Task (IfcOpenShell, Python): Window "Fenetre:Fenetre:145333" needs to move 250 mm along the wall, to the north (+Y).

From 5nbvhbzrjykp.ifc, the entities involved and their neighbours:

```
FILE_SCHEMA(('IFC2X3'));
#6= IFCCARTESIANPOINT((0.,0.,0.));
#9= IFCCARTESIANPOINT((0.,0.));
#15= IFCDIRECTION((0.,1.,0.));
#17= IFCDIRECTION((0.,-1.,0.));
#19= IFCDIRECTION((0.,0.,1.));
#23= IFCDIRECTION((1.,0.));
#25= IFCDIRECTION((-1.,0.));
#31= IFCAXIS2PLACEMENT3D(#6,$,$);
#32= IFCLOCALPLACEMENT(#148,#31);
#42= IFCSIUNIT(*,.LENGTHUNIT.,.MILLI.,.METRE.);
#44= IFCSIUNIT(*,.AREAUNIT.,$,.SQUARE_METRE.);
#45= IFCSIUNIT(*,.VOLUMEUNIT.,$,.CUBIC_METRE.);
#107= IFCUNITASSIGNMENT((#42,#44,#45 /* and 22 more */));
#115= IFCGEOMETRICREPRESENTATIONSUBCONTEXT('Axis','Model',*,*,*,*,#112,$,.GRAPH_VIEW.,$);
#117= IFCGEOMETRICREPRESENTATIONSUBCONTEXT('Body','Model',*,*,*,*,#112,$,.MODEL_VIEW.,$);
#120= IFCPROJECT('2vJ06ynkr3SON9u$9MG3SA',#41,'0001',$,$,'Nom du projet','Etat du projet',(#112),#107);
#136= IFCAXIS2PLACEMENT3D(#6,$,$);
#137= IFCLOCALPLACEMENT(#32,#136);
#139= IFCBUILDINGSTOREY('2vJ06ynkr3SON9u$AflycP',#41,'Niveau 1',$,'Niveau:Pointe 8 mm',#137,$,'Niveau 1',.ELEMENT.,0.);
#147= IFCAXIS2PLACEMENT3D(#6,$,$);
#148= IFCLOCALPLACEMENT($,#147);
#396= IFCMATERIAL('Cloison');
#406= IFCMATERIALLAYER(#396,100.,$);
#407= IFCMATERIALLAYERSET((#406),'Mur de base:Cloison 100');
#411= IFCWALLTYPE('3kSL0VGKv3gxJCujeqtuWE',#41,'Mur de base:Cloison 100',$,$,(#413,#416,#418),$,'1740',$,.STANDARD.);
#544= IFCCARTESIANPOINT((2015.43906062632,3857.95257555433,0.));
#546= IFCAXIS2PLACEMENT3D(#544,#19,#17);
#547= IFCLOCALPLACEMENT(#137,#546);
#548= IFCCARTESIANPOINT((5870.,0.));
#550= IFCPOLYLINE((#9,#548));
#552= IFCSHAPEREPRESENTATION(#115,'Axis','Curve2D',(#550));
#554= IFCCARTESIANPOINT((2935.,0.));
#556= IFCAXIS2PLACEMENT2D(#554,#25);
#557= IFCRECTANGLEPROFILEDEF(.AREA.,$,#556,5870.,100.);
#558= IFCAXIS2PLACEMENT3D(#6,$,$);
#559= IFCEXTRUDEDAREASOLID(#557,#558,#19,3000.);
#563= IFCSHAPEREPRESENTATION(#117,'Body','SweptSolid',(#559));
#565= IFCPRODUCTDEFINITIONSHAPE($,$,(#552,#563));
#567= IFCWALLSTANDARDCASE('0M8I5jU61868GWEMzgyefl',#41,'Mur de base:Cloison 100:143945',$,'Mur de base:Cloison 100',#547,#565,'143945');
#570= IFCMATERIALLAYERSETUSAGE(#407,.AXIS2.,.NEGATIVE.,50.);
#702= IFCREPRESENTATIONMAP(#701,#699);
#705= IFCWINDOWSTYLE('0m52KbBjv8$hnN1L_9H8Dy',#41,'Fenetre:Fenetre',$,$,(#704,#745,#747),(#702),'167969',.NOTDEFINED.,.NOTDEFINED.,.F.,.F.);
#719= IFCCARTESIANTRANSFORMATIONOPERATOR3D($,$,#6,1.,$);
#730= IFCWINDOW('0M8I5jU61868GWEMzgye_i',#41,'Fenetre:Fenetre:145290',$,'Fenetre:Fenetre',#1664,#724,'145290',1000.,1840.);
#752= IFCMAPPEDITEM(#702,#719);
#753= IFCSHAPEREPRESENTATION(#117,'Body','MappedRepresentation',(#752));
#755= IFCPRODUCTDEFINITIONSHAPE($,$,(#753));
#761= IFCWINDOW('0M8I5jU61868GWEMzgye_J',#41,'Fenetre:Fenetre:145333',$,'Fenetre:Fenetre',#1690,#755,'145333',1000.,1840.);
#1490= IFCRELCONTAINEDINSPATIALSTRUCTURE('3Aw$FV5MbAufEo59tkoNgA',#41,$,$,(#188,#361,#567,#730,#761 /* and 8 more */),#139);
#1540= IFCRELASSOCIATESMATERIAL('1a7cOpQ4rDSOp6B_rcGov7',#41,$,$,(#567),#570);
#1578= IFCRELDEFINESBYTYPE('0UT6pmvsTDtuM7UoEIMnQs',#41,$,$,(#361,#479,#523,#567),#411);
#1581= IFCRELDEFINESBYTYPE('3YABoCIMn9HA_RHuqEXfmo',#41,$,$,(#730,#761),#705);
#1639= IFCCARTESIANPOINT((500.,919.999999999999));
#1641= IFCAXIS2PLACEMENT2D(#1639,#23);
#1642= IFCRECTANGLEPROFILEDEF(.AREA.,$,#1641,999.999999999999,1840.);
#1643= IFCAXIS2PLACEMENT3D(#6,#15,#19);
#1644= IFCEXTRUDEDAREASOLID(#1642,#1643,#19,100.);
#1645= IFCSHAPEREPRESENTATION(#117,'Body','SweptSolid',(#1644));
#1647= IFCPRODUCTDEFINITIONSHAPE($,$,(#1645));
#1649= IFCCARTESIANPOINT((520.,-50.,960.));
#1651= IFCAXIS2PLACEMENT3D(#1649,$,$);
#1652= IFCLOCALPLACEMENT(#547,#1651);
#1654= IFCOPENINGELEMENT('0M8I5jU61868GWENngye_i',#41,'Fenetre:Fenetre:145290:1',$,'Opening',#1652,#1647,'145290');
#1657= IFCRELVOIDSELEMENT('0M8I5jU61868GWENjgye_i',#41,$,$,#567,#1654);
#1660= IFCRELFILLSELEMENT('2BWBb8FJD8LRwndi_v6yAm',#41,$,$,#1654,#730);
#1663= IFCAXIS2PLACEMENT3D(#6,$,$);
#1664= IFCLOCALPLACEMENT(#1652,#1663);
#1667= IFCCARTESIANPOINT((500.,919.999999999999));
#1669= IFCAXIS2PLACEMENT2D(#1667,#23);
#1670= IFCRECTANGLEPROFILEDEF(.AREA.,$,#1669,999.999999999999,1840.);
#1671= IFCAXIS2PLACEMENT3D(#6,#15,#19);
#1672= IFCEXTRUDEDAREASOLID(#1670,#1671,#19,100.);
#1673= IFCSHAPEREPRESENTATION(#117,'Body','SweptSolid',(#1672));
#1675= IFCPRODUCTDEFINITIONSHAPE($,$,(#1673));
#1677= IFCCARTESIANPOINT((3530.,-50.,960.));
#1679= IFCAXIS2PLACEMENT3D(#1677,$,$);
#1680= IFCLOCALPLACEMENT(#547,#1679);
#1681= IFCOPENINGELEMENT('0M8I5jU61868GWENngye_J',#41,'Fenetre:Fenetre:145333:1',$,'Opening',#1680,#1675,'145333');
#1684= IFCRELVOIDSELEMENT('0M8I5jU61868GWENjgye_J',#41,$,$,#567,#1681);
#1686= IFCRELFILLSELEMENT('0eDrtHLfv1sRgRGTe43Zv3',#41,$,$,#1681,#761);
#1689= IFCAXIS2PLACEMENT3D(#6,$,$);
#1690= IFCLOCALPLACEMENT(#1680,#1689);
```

```python
import ifcopenshell
import ifcopenshell.api.geometry
import ifcopenshell.util.placement
import ifcopenshell.util.unit

model = ifcopenshell.open("5nbvhbzrjykp.ifc")
unit_scale = ifcopenshell.util.unit.calculate_unit_scale(model)

window = model.by_guid("0M8I5jU61868GWEMzgye_J")
opening = window.FillsVoids[0].RelatingOpeningElement
wall = opening.VoidsElements[0].RelatingBuildingElement

wall_matrix = ifcopenshell.util.placement.get_local_placement(wall.ObjectPlacement)
shift = wall_matrix[:3, 0] * -0.25 / unit_scale
before = ifcopenshell.util.placement.get_local_placement(window.ObjectPlacement)[:3, 3].copy()

# The window is placed relative to its opening, so it follows when the opening moves.
matrix = ifcopenshell.util.placement.get_local_placement(opening.ObjectPlacement)
matrix[:3, 3] += shift
ifcopenshell.api.geometry.edit_object_placement(
    model, product=opening, matrix=matrix, is_si=False, should_transform_children=True
)

after = ifcopenshell.util.placement.get_local_placement(window.ObjectPlacement)[:3, 3]
print("window moved by", (after - before).round(3) + 0.0)

model.write("5nbvhbzrjykp_updated.ifc")
```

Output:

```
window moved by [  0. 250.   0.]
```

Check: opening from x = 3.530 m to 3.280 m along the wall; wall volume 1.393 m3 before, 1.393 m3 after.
